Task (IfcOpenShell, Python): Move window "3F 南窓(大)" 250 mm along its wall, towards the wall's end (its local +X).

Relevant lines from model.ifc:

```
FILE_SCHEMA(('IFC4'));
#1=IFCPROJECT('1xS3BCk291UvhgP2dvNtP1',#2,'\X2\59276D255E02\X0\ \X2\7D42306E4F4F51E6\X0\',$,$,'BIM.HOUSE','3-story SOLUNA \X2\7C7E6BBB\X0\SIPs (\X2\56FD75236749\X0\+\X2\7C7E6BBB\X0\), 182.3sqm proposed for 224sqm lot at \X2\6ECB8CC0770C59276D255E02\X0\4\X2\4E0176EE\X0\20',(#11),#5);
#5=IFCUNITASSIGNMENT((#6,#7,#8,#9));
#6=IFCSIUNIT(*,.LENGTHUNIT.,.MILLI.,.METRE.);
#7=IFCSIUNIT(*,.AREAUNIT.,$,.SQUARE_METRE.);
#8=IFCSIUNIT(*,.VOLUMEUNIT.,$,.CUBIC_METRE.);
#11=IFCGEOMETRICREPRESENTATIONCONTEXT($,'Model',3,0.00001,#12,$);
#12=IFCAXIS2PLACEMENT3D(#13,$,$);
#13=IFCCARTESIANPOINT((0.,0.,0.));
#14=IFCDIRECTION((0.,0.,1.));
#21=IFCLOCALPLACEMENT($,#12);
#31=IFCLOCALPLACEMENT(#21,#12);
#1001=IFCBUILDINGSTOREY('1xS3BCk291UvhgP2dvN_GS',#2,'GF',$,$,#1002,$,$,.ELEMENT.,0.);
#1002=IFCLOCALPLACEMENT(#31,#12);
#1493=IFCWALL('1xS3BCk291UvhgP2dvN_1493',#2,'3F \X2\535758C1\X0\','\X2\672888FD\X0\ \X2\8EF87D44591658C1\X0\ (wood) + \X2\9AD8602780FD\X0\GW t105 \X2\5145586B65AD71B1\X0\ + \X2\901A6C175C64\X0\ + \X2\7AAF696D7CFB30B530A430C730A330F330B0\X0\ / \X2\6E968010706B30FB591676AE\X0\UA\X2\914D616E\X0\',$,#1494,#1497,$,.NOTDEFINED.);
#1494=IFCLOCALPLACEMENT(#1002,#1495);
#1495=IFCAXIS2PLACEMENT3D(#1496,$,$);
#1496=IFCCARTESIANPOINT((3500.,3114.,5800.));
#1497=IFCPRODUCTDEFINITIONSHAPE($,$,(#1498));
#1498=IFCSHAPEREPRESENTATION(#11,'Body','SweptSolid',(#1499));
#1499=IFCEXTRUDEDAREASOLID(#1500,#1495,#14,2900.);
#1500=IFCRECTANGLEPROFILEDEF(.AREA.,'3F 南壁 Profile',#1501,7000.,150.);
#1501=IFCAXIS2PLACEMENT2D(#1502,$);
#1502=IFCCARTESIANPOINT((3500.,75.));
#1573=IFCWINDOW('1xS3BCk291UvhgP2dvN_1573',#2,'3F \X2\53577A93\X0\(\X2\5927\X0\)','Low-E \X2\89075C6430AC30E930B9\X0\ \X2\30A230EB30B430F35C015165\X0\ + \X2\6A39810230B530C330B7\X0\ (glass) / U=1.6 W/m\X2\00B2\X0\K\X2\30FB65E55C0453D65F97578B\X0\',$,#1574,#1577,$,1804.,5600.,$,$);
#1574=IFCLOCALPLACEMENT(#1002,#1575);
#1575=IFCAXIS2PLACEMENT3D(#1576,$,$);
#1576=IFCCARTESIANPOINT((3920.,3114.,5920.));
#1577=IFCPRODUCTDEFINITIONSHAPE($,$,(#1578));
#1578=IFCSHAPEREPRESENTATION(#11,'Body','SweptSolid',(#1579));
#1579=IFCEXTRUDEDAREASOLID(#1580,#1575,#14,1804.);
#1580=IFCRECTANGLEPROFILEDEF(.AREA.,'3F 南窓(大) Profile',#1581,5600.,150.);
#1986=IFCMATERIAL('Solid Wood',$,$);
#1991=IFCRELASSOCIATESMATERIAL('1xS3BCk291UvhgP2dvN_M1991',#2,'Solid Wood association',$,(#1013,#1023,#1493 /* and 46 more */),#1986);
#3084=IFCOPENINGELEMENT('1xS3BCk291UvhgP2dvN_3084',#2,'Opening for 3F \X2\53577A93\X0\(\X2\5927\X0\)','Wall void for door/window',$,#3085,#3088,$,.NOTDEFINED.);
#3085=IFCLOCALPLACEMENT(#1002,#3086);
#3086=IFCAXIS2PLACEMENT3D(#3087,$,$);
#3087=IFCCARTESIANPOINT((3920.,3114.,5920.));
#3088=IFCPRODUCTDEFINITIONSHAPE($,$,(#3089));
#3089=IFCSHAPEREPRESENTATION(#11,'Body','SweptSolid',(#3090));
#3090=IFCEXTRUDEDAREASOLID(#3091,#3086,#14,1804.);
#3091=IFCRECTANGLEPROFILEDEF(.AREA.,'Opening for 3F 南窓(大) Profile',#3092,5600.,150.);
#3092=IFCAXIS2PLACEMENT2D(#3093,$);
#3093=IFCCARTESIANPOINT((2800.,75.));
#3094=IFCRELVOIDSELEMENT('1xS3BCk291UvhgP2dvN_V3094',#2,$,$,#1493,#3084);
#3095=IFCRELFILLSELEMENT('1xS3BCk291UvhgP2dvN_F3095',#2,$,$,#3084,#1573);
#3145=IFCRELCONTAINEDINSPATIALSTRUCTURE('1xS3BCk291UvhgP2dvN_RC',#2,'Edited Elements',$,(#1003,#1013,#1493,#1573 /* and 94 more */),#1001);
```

```python
import ifcopenshell
import ifcopenshell.api.geometry
import ifcopenshell.util.placement
import ifcopenshell.util.unit

model = ifcopenshell.open("model.ifc")
unit_scale = ifcopenshell.util.unit.calculate_unit_scale(model)

window = model.by_guid("1xS3BCk291UvhgP2dvN_1573")
opening = window.FillsVoids[0].RelatingOpeningElement
wall = opening.VoidsElements[0].RelatingBuildingElement

wall_matrix = ifcopenshell.util.placement.get_local_placement(wall.ObjectPlacement)
shift = wall_matrix[:3, 0] * 0.25 / unit_scale
before = ifcopenshell.util.placement.get_local_placement(window.ObjectPlacement)[:3, 3].copy()

# The window is not placed relative to its opening, so move both.
for product in (opening, window):
    matrix = ifcopenshell.util.placement.get_local_placement(product.ObjectPlacement)
    matrix[:3, 3] += shift
    ifcopenshell.api.geometry.edit_object_placement(model, product=product, matrix=matrix, is_si=False)

after = ifcopenshell.util.placement.get_local_placement(window.ObjectPlacement)[:3, 3]
print("window moved by", (after - before).round(3) + 0.0)

model.write("model_rev.ifc")
```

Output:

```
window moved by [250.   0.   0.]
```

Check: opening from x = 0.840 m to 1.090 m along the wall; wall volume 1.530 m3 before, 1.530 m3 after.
